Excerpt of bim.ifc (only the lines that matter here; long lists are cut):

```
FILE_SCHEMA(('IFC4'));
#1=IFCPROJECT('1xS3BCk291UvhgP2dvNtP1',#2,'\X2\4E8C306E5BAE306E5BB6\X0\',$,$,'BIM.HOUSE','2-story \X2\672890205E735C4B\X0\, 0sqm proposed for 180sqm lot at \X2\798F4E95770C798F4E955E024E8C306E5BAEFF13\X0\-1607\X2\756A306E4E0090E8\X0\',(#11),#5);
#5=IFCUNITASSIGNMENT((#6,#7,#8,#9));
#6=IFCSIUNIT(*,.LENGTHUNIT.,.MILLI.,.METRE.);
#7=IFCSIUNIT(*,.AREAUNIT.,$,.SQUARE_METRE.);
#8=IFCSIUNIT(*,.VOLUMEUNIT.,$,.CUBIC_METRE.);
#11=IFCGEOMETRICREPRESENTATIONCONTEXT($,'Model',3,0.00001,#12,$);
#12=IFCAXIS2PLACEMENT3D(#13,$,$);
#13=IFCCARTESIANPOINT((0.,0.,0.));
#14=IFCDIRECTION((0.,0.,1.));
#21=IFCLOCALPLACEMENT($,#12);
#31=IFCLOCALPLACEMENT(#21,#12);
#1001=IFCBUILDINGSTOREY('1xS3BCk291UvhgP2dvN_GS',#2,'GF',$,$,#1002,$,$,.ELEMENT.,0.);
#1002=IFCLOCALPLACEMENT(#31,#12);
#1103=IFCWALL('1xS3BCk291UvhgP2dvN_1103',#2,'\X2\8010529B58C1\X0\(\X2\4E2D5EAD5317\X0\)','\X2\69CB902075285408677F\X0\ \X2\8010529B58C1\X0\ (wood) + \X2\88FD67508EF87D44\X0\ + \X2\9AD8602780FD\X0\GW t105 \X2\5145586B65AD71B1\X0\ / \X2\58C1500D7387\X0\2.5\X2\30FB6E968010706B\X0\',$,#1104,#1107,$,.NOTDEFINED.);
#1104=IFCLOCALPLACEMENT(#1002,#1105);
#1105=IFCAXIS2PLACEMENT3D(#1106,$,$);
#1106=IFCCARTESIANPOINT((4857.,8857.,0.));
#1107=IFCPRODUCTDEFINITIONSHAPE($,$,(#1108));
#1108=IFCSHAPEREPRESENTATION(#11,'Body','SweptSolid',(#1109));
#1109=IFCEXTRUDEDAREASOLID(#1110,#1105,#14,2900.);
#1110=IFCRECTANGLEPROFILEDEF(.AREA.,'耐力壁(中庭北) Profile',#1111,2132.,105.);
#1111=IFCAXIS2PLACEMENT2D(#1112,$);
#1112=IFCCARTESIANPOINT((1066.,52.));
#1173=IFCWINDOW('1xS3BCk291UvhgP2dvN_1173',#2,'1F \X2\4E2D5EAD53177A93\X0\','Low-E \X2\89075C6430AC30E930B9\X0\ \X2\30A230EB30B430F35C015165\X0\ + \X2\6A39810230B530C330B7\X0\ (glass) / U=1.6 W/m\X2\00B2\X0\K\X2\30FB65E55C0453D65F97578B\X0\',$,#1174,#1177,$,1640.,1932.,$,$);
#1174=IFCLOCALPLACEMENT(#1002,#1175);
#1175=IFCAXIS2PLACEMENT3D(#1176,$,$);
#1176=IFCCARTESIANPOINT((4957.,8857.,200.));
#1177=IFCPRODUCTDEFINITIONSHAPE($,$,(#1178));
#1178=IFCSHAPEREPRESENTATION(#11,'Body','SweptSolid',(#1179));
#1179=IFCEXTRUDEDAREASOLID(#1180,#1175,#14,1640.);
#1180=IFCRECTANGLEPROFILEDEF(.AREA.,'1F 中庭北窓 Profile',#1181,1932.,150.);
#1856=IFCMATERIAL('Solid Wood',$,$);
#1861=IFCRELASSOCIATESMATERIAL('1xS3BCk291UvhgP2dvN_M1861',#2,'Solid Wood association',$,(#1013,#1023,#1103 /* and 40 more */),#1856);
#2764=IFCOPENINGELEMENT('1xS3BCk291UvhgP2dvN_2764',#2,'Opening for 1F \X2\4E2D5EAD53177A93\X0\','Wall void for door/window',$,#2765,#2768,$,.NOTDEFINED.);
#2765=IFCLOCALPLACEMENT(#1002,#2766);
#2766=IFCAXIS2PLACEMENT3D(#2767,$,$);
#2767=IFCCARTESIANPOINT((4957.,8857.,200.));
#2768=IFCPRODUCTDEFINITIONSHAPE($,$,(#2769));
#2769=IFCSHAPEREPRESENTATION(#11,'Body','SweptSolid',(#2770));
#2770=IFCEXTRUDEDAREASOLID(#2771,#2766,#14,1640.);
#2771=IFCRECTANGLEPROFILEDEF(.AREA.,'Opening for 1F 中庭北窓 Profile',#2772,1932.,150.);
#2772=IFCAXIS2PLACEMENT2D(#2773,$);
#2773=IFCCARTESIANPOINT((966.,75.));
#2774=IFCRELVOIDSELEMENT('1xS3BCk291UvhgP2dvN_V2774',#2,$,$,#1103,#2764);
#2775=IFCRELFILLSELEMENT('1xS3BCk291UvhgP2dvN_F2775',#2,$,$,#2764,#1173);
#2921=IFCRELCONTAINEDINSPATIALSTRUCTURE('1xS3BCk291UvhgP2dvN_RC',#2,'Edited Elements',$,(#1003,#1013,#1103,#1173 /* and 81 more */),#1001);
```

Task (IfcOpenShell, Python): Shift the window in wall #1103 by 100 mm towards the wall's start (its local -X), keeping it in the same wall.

```python
import ifcopenshell
import ifcopenshell.api.geometry
import ifcopenshell.util.placement
import ifcopenshell.util.unit

model = ifcopenshell.open("bim.ifc")
unit_scale = ifcopenshell.util.unit.calculate_unit_scale(model)

window = model.by_guid("1xS3BCk291UvhgP2dvN_1173")
opening = window.FillsVoids[0].RelatingOpeningElement
wall = opening.VoidsElements[0].RelatingBuildingElement

wall_matrix = ifcopenshell.util.placement.get_local_placement(wall.ObjectPlacement)
shift = wall_matrix[:3, 0] * -0.1 / unit_scale
before = ifcopenshell.util.placement.get_local_placement(window.ObjectPlacement)[:3, 3].copy()

# The window is not placed relative to its opening, so move both.
for product in (opening, window):
    matrix = ifcopenshell.util.placement.get_local_placement(product.ObjectPlacement)
    matrix[:3, 3] += shift
    ifcopenshell.api.geometry.edit_object_placement(model, product=product, matrix=matrix, is_si=False)

after = ifcopenshell.util.placement.get_local_placement(window.ObjectPlacement)[:3, 3]
print("window moved by", (after - before).round(3) + 0.0)

model.write("bim_rev.ifc")
```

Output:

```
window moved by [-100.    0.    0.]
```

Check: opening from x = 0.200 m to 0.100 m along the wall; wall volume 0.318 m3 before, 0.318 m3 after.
